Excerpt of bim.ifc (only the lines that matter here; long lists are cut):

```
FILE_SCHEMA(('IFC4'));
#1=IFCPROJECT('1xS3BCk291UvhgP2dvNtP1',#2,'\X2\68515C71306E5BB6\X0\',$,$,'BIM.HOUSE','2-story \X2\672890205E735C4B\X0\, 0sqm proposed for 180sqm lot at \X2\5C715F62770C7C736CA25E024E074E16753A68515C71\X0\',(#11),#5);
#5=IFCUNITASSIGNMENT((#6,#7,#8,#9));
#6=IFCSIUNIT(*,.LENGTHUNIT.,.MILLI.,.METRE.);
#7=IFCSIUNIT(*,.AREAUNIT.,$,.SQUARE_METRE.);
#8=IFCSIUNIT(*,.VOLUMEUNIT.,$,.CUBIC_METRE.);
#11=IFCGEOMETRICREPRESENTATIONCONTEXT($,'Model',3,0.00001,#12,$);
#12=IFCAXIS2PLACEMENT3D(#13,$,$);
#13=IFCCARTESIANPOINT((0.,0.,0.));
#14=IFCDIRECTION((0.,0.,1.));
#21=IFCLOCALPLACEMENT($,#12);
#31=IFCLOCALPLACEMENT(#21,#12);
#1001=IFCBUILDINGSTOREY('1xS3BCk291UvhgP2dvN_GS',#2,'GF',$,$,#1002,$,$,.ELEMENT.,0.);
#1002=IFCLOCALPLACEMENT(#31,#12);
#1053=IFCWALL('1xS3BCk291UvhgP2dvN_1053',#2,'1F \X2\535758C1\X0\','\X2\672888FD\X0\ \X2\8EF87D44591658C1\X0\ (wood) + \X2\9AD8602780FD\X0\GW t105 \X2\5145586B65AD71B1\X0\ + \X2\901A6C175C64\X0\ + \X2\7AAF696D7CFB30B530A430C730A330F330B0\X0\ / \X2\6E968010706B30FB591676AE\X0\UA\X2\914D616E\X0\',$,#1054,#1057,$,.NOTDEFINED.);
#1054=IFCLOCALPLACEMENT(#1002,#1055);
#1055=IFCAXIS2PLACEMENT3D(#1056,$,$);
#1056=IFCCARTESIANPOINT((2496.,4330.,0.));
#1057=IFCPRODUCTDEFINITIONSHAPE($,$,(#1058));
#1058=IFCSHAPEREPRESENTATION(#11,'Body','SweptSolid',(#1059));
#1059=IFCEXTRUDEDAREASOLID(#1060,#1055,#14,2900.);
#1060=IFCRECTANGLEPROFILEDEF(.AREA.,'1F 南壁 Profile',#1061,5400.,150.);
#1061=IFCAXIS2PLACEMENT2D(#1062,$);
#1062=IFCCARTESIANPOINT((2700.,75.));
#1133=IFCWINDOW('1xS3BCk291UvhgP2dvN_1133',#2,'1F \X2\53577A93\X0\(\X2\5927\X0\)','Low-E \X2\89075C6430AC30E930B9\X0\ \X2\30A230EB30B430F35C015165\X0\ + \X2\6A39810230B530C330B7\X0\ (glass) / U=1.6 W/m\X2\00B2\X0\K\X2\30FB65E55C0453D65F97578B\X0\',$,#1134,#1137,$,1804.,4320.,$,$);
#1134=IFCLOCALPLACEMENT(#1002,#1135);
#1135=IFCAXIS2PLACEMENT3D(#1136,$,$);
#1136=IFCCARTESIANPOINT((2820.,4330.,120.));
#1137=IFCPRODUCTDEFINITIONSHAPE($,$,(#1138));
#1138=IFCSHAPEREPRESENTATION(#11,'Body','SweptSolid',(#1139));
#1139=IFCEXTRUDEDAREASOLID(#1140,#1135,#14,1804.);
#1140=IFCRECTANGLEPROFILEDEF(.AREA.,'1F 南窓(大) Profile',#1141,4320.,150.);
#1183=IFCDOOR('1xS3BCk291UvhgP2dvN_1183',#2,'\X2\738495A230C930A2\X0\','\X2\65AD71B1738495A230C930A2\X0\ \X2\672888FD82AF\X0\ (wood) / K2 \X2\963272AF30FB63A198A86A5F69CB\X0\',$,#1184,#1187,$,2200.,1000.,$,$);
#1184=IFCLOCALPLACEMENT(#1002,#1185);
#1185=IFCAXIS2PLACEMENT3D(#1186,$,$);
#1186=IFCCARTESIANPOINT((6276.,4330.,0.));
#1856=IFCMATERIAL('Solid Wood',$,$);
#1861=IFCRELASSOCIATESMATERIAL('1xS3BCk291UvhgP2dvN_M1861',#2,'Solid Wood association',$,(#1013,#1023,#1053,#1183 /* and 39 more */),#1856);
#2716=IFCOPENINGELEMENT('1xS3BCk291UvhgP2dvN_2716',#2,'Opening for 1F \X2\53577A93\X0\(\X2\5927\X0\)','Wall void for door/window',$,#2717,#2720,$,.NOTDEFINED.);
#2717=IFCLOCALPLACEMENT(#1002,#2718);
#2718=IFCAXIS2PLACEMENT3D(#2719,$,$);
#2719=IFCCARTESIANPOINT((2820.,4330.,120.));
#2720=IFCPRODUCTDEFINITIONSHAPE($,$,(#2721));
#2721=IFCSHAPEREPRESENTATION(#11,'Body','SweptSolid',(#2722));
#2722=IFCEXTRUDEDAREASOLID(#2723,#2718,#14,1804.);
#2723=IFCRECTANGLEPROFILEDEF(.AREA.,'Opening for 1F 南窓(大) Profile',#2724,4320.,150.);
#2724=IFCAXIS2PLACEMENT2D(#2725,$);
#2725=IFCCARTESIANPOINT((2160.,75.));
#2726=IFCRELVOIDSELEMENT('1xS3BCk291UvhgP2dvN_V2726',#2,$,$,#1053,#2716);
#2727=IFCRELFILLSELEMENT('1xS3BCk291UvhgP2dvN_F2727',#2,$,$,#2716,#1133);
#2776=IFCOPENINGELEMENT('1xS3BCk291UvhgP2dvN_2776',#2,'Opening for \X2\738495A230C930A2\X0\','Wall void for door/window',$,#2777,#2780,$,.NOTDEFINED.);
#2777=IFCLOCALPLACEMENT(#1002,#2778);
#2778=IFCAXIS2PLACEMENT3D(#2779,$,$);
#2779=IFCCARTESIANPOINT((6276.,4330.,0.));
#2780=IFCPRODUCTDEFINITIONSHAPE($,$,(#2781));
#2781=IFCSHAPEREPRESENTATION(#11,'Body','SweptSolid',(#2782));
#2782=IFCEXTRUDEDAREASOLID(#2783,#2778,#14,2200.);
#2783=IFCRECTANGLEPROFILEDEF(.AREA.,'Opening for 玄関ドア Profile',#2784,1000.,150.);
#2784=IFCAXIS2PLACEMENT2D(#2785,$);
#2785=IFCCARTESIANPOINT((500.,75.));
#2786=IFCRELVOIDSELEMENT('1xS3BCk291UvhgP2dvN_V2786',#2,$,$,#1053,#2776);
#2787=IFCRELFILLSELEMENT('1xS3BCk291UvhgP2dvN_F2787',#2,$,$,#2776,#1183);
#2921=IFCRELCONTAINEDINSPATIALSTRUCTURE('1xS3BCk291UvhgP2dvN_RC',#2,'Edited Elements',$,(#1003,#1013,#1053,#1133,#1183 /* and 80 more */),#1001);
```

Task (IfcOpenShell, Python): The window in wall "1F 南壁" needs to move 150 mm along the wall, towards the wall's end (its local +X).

```python
import ifcopenshell
import ifcopenshell.api.geometry
import ifcopenshell.util.placement
import ifcopenshell.util.unit

model = ifcopenshell.open("bim.ifc")
unit_scale = ifcopenshell.util.unit.calculate_unit_scale(model)

window = model.by_guid("1xS3BCk291UvhgP2dvN_1133")
opening = window.FillsVoids[0].RelatingOpeningElement
wall = opening.VoidsElements[0].RelatingBuildingElement

wall_matrix = ifcopenshell.util.placement.get_local_placement(wall.ObjectPlacement)
shift = wall_matrix[:3, 0] * 0.15 / unit_scale
before = ifcopenshell.util.placement.get_local_placement(window.ObjectPlacement)[:3, 3].copy()

# The window is not placed relative to its opening, so move both.
for product in (opening, window):
    matrix = ifcopenshell.util.placement.get_local_placement(product.ObjectPlacement)
    matrix[:3, 3] += shift
    ifcopenshell.api.geometry.edit_object_placement(model, product=product, matrix=matrix, is_si=False)

after = ifcopenshell.util.placement.get_local_placement(window.ObjectPlacement)[:3, 3]
print("window moved by", (after - before).round(3) + 0.0)

model.write("bim_rev.ifc")
```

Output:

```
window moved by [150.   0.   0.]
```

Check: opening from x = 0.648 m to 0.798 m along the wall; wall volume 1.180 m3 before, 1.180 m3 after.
